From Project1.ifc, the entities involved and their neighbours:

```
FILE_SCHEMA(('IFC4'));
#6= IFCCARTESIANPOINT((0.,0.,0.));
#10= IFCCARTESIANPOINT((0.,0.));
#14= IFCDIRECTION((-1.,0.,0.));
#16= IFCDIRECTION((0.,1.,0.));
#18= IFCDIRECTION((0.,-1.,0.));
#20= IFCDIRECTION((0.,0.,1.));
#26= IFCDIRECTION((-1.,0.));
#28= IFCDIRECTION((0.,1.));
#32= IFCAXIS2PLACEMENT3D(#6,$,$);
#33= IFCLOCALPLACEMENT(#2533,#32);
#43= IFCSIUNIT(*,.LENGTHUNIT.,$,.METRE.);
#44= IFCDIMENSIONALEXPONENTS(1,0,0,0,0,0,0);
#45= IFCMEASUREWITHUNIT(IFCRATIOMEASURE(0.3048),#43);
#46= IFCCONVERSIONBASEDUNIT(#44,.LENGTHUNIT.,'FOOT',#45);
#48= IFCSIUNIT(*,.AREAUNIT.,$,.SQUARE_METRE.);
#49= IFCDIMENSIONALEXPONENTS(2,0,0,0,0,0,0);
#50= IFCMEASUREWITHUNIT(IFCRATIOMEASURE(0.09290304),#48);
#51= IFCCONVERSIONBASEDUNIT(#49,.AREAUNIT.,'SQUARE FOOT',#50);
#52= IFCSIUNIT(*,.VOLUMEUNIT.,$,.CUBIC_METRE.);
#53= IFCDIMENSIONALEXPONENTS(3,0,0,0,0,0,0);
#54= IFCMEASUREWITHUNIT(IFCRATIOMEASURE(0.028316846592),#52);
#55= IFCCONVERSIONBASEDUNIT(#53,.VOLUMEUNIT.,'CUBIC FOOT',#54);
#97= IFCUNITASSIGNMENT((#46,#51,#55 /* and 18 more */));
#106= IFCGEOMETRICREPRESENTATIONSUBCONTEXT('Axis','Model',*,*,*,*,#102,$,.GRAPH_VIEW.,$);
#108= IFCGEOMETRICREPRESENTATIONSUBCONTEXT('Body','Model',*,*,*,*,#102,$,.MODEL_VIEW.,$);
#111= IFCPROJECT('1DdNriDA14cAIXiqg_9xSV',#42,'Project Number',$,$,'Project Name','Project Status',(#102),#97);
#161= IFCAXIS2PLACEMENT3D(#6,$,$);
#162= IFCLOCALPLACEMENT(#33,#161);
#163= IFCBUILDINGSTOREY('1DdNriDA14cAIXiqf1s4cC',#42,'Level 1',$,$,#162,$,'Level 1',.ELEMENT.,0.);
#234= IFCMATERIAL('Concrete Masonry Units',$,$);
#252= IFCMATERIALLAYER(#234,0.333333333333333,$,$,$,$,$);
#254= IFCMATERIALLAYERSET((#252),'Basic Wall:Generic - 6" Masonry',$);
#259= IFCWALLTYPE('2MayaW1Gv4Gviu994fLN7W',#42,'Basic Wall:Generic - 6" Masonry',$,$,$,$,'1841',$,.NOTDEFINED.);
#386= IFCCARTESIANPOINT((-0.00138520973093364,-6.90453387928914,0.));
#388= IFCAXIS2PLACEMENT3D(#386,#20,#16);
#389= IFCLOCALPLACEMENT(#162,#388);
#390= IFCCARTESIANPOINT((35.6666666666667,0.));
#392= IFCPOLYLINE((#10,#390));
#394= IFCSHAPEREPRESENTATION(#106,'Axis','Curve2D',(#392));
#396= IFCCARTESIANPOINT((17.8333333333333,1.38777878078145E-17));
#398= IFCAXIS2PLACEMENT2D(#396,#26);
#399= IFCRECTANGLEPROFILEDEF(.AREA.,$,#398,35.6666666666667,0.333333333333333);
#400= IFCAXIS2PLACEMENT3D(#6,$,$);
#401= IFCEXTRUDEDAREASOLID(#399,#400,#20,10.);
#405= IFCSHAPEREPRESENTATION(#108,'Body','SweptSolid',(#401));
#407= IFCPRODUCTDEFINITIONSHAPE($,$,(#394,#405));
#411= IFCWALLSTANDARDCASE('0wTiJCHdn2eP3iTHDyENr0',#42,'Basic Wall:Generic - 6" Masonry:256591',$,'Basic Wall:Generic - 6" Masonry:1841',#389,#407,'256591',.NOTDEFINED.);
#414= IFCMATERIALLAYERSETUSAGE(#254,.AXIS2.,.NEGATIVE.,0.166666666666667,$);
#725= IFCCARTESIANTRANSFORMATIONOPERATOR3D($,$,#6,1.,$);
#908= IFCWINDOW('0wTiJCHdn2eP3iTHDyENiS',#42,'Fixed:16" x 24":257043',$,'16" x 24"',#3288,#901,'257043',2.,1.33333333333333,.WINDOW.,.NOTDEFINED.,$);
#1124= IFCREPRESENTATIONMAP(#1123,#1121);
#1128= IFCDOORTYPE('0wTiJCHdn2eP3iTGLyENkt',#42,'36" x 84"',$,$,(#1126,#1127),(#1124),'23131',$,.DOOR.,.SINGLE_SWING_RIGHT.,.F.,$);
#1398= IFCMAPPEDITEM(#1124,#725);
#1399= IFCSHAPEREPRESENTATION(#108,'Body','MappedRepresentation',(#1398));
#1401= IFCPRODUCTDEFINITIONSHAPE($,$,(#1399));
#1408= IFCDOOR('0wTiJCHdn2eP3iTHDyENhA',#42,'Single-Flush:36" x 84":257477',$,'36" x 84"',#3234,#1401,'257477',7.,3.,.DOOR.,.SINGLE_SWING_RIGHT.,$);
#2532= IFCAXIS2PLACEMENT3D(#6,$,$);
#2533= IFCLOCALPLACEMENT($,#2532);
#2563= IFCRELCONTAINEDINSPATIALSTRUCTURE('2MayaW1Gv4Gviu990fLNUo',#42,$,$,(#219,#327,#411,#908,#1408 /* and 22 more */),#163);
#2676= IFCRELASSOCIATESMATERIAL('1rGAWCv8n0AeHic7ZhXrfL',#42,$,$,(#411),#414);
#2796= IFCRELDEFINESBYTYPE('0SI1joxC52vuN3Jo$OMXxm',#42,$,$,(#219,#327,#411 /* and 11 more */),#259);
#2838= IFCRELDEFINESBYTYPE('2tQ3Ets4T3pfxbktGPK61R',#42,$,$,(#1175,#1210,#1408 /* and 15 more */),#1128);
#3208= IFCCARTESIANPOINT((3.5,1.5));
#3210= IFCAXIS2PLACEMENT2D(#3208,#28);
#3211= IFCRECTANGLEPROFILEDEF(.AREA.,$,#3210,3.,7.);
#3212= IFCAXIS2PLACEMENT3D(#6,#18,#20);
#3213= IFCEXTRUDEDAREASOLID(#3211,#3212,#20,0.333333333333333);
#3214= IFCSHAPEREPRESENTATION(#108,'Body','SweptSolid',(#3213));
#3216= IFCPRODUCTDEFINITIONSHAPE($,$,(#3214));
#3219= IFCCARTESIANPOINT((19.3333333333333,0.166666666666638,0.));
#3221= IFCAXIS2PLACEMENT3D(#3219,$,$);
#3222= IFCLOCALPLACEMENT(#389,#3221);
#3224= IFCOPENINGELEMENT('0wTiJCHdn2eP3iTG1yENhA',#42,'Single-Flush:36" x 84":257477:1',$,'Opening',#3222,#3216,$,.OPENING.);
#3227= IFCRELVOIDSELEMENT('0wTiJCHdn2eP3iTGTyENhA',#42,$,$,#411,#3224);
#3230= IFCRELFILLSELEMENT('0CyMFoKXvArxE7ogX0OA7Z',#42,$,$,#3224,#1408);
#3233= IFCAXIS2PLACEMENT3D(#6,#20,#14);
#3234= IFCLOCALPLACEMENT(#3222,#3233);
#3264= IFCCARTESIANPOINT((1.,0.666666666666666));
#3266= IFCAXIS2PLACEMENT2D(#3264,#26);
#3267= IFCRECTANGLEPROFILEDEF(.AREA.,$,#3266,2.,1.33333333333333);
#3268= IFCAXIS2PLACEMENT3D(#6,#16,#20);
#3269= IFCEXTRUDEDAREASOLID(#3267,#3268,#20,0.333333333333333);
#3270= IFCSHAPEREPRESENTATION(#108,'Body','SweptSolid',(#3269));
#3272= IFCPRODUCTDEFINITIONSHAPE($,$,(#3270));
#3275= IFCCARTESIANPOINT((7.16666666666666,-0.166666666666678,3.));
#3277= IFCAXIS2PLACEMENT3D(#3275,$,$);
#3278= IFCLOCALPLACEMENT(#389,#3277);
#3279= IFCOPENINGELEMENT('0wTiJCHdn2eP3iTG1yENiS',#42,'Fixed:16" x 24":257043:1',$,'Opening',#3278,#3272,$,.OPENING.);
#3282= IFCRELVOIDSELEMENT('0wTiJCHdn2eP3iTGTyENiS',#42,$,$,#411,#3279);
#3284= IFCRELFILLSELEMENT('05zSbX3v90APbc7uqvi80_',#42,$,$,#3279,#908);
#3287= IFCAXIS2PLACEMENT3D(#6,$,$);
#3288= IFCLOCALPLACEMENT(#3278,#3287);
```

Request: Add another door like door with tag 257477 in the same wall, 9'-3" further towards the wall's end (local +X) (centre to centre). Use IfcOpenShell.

```python
import ifcopenshell
import ifcopenshell.api.feature
import ifcopenshell.api.geometry
import ifcopenshell.api.root
import ifcopenshell.geom
import ifcopenshell.util.element
import ifcopenshell.util.placement
import ifcopenshell.util.shape
import ifcopenshell.util.unit

model = ifcopenshell.open("Project1.ifc")
unit_scale = ifcopenshell.util.unit.calculate_unit_scale(model)
settings = ifcopenshell.geom.settings()


def volume(element):
    """Net volume in cubic metres, openings subtracted."""
    shape = ifcopenshell.geom.create_shape(settings, element)
    return ifcopenshell.util.shape.get_volume(shape.geometry)


def reuse_history(source, copy):
    """copy_class also copies each property set's owner history, people and application; keep the originals."""
    for rel in copy.IsDefinedBy:
        if rel.is_a("IfcRelDefinesByProperties") and (history := rel.RelatingPropertyDefinition.OwnerHistory):
            rel.RelatingPropertyDefinition.OwnerHistory = source.OwnerHistory
            ifcopenshell.util.element.remove_deep2(model, history)


door = model.by_guid("0wTiJCHdn2eP3iTHDyENhA")
opening = door.FillsVoids[0].RelatingOpeningElement
wall = opening.VoidsElements[0].RelatingBuildingElement
before = volume(wall)
shift = ifcopenshell.util.placement.get_local_placement(wall.ObjectPlacement)[:3, 0] * 111 * 0.0254 / unit_scale

# copy_class copies the void relationship, type, container and properties, but no geometry.
new_opening = ifcopenshell.api.root.copy_class(model, product=opening)
new_opening.Representation = ifcopenshell.util.element.copy_deep(
    model, opening.Representation, exclude=["IfcGeometricRepresentationContext", "IfcRepresentationMap"]
)
new_opening.Name = 'Single-Flush:36" x 84"'
new_door = ifcopenshell.api.root.copy_class(model, product=door)
new_door.Representation = ifcopenshell.util.element.copy_deep(
    model, door.Representation, exclude=["IfcGeometricRepresentationContext", "IfcRepresentationMap"]
)
new_door.Name = 'Single-Flush:36" x 84"'
new_door.Tag = None
reuse_history(door, new_door)
ifcopenshell.api.feature.add_filling(model, opening=new_opening, element=new_door)

for old, new in ((opening, new_opening), (door, new_door)):
    matrix = ifcopenshell.util.placement.get_local_placement(old.ObjectPlacement)
    matrix[:3, 3] += shift
    ifcopenshell.api.geometry.edit_object_placement(model, product=new, matrix=matrix, is_si=False)

after = volume(wall)

print(f"wall volume {before:.3f} -> {after:.3f} m3")

model.write("Project1_v2.ifc")
```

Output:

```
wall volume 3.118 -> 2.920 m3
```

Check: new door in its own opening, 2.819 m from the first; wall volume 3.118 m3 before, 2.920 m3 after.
